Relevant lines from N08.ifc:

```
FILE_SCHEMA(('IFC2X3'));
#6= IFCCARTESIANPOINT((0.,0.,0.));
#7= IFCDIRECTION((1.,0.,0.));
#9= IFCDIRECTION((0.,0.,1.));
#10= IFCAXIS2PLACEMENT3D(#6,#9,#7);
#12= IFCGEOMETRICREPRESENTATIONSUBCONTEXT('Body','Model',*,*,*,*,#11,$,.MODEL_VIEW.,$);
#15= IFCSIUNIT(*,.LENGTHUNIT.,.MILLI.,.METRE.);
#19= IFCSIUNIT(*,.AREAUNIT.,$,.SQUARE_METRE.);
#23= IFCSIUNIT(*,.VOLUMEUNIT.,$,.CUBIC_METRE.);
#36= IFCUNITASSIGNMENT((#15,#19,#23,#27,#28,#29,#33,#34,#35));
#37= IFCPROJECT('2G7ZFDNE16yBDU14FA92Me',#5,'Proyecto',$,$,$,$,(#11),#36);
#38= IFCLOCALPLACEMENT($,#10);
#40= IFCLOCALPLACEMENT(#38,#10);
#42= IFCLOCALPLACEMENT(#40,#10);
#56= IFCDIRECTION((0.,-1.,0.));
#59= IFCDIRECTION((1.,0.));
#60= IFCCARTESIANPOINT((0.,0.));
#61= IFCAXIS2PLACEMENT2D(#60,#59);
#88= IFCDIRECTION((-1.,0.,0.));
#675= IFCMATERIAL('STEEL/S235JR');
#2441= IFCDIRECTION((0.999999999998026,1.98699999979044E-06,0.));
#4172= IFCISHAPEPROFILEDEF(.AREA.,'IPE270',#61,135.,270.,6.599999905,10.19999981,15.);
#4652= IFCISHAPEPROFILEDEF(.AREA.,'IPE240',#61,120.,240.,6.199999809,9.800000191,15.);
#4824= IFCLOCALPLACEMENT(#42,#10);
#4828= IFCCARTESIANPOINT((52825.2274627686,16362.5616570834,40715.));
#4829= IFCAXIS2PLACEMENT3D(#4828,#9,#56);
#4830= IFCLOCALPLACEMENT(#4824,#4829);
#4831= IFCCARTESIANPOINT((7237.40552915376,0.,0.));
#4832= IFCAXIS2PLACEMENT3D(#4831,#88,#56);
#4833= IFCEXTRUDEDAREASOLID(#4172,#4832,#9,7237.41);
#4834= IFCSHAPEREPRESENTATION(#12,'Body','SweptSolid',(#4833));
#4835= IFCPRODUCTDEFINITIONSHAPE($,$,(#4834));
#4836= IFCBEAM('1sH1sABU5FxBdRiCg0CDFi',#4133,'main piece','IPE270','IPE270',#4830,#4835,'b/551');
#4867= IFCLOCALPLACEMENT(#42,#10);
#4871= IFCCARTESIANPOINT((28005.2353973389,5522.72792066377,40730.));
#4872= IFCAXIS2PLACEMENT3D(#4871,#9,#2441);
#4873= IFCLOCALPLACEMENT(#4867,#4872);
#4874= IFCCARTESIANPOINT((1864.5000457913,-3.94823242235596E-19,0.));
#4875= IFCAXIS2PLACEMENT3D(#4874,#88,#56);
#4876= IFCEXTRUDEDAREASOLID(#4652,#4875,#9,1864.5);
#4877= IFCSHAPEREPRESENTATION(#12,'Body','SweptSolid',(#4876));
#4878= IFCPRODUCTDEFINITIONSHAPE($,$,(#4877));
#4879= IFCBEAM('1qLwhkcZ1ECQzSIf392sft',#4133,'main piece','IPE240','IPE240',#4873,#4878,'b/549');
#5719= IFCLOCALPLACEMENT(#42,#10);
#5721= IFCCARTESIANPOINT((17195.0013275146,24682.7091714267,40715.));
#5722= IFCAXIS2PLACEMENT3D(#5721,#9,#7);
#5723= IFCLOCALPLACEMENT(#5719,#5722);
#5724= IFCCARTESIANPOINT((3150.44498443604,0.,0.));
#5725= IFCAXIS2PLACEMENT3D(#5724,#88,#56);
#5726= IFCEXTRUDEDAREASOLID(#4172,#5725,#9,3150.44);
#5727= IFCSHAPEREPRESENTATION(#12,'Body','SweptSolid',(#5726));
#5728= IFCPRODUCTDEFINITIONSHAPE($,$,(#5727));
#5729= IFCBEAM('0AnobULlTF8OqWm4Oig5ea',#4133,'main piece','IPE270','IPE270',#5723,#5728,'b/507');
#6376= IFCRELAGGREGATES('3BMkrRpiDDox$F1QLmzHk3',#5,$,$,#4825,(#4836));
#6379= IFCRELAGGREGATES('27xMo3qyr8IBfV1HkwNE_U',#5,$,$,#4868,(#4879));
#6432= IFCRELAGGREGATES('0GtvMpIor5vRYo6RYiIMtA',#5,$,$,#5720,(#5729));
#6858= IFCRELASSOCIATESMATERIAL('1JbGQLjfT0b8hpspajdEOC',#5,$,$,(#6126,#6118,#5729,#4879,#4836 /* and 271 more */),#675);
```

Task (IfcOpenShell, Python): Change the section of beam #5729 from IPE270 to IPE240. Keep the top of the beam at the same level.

```python
import ifcopenshell
import ifcopenshell.util.element
import ifcopenshell.util.representation

model = ifcopenshell.open("N08.ifc")

member = model.by_id(5729)
source = next(p for p in model.by_type("IfcIShapeProfileDef") if p.ProfileName == "IPE240")

body = ifcopenshell.util.representation.get_representation(member, "Model", "Body")
solid = body.Items[0]
old_profile = solid.SweptArea

# Copy the section's sizes but keep this member's own profile position.
profile = ifcopenshell.util.element.copy(model, source)
# Profiles are centred, so shift by half the change in depth to hold the top.
shift = (old_profile.OverallDepth - profile.OverallDepth) / 2
x, y = old_profile.Position.Location.Coordinates
up = (0.0, 1.0)  # upwards, in the solid's own plane
location = model.createIfcCartesianPoint((x + up[0] * shift, y + up[1] * shift))
profile.Position = model.createIfcAxis2Placement2D(location, old_profile.Position.RefDirection)
solid.SweptArea = profile
if not model.get_total_inverses(old_profile):
    ifcopenshell.util.element.remove_deep2(model, old_profile)
member.Description = member.Description.replace("IPE270", "IPE240")
member.ObjectType = member.ObjectType.replace("IPE270", "IPE240")

print(solid.SweptArea)

model.write("N08_updated.ifc")
```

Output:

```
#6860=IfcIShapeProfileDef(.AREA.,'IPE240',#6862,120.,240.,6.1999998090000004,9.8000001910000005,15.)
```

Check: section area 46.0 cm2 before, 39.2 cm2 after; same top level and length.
